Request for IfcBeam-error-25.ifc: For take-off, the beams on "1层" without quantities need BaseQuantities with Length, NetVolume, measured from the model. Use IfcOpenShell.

First a look at what the model holds.

```python
import ifcopenshell
import ifcopenshell.util.element
import ifcopenshell.util.unit

model = ifcopenshell.open("IfcBeam-error-25.ifc")
print(model.schema)
for unit_type in ("LENGTHUNIT", "AREAUNIT", "VOLUMEUNIT"):
    print(unit_type, ifcopenshell.util.unit.calculate_unit_scale(model, unit_type))
storey = next(s for s in model.by_type("IfcBuildingStorey") if s.Name == "1层")
beams = [e for e in ifcopenshell.util.element.get_decomposition(storey) if e.is_a("IfcBeam")]
for e in sorted(beams, key=lambda e: e.id()):
    print(e.id(), e.is_a(), e.Name, list(ifcopenshell.util.element.get_psets(e, qtos_only=True)), sep=" | ")
```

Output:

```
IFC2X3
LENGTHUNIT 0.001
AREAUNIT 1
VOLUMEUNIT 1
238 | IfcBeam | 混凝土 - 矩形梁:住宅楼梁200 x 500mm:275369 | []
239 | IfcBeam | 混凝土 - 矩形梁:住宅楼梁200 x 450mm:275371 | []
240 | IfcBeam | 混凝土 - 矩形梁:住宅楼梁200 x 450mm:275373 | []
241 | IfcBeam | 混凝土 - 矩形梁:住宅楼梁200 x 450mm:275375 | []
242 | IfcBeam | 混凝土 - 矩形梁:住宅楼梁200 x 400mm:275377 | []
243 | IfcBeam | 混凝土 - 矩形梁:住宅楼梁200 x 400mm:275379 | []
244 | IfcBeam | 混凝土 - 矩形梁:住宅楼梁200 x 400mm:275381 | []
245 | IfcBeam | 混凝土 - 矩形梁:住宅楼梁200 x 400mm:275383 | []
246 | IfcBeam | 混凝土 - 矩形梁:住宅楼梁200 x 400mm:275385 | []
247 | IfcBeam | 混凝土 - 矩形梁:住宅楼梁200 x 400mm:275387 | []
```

```python
import ifcopenshell
import ifcopenshell.api.pset
import ifcopenshell.geom
import ifcopenshell.util.element
import ifcopenshell.util.shape
import ifcopenshell.util.unit

model = ifcopenshell.open("IfcBeam-error-25.ifc")
unit_scale = ifcopenshell.util.unit.calculate_unit_scale(model)
volume_scale = ifcopenshell.util.unit.calculate_unit_scale(model, "VOLUMEUNIT")
settings = ifcopenshell.geom.settings()

storey = next(s for s in model.by_type("IfcBuildingStorey") if s.Name == "1层")
beams = [e for e in ifcopenshell.util.element.get_decomposition(storey) if e.is_a("IfcBeam")]

for e in sorted(beams, key=lambda e: e.id()):
    if ifcopenshell.util.element.get_psets(e, qtos_only=True, should_inherit=False):
        continue
    # Geometry comes back in metres, in the element's own axes.
    shape = ifcopenshell.geom.create_shape(settings, e)
    values = {
        "Length": ifcopenshell.util.shape.get_max_xyz(shape.geometry) / unit_scale,
        "NetVolume": ifcopenshell.util.shape.get_volume(shape.geometry) / volume_scale,
    }
    qto = ifcopenshell.api.pset.add_qto(model, product=e, name="BaseQuantities")
    ifcopenshell.api.pset.edit_qto(model, qto=qto, properties=values)
    print(e.id(), {k: round(v, 3) for k, v in values.items()})

model.write("IfcBeam-error-25_edited.ifc")
```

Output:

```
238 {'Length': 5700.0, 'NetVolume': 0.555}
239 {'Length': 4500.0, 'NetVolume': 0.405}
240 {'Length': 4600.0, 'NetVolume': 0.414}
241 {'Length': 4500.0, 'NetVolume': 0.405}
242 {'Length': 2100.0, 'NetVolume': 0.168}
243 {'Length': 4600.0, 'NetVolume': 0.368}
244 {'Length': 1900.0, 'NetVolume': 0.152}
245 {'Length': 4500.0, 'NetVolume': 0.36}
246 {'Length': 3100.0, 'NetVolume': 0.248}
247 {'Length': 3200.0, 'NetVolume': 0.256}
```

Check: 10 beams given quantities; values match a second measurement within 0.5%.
